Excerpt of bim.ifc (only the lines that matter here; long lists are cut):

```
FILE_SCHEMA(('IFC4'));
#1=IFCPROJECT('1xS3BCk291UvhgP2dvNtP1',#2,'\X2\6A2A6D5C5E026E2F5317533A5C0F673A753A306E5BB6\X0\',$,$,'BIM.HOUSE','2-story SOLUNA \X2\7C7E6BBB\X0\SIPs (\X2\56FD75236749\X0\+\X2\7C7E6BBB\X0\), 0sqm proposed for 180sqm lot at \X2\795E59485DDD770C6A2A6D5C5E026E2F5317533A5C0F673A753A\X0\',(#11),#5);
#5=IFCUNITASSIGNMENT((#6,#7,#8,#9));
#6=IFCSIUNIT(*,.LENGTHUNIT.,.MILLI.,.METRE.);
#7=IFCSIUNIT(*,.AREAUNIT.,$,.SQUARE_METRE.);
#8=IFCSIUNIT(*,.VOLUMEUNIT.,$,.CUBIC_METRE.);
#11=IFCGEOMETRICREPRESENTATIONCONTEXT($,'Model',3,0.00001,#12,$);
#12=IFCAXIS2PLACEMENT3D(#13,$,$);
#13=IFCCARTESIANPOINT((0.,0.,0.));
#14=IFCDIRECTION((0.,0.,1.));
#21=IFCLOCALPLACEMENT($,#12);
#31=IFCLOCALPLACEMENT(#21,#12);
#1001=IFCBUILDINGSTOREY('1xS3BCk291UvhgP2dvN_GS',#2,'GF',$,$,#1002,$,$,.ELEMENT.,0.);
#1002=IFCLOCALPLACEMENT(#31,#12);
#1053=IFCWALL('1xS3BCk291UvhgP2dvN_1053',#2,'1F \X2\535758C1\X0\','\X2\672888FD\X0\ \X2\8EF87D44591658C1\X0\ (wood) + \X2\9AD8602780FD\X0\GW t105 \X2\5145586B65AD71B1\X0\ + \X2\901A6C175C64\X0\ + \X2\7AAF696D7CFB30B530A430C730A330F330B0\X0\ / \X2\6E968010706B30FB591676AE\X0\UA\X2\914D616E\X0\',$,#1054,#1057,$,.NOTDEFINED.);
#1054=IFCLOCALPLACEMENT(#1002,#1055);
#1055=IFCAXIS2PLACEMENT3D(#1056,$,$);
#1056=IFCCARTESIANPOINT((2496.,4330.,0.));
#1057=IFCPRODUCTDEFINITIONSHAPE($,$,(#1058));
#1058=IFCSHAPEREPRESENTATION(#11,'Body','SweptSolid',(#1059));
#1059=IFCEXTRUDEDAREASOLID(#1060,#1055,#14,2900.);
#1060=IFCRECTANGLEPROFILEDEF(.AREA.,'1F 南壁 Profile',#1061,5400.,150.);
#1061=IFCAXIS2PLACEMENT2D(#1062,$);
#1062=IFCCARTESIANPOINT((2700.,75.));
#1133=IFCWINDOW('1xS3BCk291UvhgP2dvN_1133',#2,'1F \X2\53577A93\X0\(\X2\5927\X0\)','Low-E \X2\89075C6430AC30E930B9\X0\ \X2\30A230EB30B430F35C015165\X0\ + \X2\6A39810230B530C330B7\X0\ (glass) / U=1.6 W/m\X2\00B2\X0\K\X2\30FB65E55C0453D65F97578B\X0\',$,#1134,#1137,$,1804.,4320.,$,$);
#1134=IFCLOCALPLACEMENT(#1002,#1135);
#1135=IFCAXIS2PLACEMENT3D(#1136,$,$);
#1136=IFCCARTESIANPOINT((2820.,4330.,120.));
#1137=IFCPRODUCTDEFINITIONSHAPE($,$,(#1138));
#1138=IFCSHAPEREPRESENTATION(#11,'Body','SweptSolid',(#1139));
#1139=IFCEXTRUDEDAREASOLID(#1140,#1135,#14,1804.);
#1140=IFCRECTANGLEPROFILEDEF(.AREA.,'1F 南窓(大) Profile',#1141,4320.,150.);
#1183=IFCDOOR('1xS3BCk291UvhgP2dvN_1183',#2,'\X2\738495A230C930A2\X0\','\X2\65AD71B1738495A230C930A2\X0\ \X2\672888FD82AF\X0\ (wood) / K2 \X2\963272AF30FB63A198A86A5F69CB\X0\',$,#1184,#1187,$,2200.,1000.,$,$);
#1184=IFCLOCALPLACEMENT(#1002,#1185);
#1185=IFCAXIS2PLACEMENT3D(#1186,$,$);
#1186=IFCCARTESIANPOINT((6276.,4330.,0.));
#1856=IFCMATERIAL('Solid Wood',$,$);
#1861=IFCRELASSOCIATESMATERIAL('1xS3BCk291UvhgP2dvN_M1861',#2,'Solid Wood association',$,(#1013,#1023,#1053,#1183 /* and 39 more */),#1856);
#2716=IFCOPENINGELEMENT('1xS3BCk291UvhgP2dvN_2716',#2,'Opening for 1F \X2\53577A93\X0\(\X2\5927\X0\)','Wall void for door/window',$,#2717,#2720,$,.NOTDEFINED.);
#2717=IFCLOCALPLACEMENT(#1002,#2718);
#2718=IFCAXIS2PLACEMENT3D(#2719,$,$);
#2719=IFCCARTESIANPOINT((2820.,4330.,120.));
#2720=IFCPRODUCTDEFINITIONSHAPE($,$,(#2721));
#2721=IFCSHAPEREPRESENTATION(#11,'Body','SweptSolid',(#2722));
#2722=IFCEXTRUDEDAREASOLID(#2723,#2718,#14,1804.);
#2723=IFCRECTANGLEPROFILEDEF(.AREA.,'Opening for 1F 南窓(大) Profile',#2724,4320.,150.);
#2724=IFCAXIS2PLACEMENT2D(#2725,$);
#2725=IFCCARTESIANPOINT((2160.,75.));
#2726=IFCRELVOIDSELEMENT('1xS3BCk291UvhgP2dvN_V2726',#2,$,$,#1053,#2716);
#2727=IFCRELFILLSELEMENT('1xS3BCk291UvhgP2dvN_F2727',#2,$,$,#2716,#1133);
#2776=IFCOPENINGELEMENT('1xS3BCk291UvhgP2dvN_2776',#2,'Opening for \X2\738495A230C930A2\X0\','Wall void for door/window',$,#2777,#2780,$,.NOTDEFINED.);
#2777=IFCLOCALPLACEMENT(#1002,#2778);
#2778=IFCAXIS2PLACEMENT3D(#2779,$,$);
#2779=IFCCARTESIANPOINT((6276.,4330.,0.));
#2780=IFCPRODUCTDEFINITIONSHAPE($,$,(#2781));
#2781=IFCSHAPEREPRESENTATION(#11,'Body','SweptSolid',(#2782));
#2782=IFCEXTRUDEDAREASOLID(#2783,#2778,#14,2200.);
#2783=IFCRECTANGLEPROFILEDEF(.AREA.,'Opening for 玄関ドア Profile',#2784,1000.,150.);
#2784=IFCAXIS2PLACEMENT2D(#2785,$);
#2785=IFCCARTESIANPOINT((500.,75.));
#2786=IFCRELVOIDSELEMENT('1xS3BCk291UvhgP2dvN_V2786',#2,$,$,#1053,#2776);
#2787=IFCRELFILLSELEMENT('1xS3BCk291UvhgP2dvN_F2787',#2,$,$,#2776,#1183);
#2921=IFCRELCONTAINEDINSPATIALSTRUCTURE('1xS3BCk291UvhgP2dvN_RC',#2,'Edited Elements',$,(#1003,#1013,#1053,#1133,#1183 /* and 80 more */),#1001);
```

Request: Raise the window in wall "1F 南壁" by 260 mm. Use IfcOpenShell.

```python
import numpy as np
import ifcopenshell
import ifcopenshell.api.geometry
import ifcopenshell.util.placement
import ifcopenshell.util.unit

model = ifcopenshell.open("bim.ifc")
unit_scale = ifcopenshell.util.unit.calculate_unit_scale(model)

window = model.by_guid("1xS3BCk291UvhgP2dvN_1133")
opening = window.FillsVoids[0].RelatingOpeningElement
dz = 0.26 / unit_scale

shift = np.array([0.0, 0.0, dz])
# The window is not placed relative to its opening, so move both.
for product in (opening, window):
    matrix = ifcopenshell.util.placement.get_local_placement(product.ObjectPlacement)
    matrix[:3, 3] += shift
    ifcopenshell.api.geometry.edit_object_placement(model, product=product, matrix=matrix, is_si=False)

print(f"moved by {dz * unit_scale:+.3f} m")

model.write("bim_updated.ifc")
```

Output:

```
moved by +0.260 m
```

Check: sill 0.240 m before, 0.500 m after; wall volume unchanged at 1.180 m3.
